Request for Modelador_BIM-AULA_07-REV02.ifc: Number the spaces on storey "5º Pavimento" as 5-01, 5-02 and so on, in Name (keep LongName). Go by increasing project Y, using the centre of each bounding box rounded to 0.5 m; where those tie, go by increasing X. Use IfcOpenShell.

First a look at what the model holds.

```python
import ifcopenshell
import ifcopenshell.util.element
import ifcopenshell.util.placement

model = ifcopenshell.open("Modelador_BIM-AULA_07-REV02.ifc")
print(model.schema)
storey = next(s for s in model.by_type("IfcBuildingStorey") if s.Name == "5º Pavimento")
spaces = [e for e in ifcopenshell.util.element.get_decomposition(storey) if e.is_a("IfcSpace")]
for e in sorted(spaces, key=lambda e: e.id()):
    origin = ifcopenshell.util.placement.get_local_placement(e.ObjectPlacement)[:3, 3]
    print(e.id(), e.Name, e.LongName, origin.round(2) + 0.0, sep=" | ")
```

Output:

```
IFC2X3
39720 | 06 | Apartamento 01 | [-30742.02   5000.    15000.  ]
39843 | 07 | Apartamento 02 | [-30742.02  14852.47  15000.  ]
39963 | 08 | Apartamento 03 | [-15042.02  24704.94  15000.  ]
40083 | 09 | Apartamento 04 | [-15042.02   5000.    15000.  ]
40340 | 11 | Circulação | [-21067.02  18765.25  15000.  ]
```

```python
import ifcopenshell
import ifcopenshell.geom
import ifcopenshell.util.element
import ifcopenshell.util.shape

model = ifcopenshell.open("Modelador_BIM-AULA_07-REV02.ifc")
settings = ifcopenshell.geom.settings()
settings.set("use-world-coords", True)


def centre(element):
    shape = ifcopenshell.geom.create_shape(settings, element)
    return ifcopenshell.util.shape.get_bbox_centroid(shape.geometry)


storey = next(s for s in model.by_type("IfcBuildingStorey") if s.Name == "5º Pavimento")
spaces = [e for e in ifcopenshell.util.element.get_decomposition(storey) if e.is_a("IfcSpace")]

# Insertion points can sit at a corner or the storey origin, so sort by the geometry (in metres).
centres = {e: centre(e) for e in spaces}
spaces.sort(key=lambda e: (round(centres[e][1] / 0.5), centres[e][0]))

for i, e in enumerate(spaces, start=1):
    number = f"5-{i:02d}"
    e.Name = number
    print(e.id(), number)

model.write("Modelador_BIM-AULA_07-REV02_updated.ifc")
```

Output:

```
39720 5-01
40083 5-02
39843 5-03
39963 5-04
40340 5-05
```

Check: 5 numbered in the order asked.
